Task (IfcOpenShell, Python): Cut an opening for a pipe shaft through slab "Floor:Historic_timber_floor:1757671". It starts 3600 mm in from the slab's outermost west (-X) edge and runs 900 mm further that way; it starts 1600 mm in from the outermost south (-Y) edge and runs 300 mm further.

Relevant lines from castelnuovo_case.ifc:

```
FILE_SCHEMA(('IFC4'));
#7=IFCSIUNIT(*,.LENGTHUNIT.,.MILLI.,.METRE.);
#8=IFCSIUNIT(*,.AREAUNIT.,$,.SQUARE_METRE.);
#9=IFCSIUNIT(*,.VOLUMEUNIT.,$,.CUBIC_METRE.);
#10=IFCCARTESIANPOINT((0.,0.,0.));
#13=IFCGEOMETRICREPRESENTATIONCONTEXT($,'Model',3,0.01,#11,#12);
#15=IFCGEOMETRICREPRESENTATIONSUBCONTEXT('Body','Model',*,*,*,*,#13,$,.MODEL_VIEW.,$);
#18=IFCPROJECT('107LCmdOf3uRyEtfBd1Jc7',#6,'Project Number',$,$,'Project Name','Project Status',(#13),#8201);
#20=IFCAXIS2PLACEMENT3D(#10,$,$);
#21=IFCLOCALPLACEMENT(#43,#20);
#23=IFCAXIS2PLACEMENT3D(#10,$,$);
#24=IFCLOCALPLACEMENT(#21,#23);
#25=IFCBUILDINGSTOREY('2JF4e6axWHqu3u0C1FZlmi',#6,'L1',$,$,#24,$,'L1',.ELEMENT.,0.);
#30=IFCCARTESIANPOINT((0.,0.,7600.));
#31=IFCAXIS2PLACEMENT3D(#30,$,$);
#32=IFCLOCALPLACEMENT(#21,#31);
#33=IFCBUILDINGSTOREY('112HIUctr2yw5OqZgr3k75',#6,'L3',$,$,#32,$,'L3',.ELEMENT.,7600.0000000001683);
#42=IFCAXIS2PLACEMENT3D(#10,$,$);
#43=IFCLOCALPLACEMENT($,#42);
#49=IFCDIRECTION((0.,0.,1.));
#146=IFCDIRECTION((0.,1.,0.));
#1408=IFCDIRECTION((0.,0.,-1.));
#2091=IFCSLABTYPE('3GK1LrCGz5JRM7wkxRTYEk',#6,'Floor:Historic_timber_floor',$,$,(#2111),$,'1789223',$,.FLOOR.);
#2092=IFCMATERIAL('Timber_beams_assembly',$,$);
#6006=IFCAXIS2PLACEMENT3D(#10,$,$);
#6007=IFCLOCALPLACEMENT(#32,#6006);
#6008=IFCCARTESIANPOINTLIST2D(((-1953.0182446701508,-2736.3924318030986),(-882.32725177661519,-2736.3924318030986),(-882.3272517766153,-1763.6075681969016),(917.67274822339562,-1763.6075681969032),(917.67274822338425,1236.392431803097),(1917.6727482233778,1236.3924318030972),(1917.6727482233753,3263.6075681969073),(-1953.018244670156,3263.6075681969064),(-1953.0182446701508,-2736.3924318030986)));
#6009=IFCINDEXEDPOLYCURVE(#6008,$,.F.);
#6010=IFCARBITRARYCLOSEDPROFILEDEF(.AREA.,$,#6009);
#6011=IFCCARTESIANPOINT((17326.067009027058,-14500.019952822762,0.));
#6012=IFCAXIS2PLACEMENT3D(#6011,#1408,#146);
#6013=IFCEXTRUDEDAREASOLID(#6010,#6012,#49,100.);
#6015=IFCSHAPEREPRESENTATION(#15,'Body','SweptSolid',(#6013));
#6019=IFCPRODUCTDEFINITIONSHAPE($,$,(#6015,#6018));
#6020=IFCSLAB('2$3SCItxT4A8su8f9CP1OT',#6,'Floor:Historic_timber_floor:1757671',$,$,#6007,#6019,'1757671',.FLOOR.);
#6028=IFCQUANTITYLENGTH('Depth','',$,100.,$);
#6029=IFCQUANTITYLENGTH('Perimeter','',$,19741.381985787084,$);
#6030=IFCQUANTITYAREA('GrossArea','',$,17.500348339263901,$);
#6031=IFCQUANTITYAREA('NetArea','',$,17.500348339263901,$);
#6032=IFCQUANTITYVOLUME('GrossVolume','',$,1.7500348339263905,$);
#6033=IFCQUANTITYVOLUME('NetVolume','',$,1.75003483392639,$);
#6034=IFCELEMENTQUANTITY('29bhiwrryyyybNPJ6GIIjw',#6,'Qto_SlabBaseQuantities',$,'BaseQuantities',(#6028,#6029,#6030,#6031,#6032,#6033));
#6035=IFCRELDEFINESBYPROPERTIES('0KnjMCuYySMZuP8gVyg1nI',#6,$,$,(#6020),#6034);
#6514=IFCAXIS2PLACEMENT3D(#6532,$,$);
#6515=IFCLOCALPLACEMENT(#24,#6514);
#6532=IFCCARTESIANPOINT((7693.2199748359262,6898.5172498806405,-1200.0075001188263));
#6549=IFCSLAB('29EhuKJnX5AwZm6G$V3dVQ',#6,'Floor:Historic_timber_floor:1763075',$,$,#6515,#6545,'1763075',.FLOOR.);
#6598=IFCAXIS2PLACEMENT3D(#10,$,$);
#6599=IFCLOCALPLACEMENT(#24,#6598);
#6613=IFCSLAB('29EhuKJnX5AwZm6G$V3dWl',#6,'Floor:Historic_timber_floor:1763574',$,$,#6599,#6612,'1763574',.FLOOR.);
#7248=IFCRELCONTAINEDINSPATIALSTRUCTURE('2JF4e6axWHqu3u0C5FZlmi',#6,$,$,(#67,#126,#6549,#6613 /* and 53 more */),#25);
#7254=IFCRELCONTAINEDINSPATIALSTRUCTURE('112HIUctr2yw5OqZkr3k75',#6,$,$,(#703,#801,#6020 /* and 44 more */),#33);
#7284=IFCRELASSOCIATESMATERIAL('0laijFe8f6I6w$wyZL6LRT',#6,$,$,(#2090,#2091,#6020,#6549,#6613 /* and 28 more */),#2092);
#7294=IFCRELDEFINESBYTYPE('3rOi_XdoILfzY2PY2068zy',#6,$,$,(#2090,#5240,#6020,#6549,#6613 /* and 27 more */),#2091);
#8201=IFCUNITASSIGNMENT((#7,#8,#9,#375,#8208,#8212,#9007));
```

```python
import numpy as np
import ifcopenshell
import ifcopenshell.api.feature
import ifcopenshell.api.geometry
import ifcopenshell.api.pset
import ifcopenshell.api.root
import ifcopenshell.geom
import ifcopenshell.util.element
import ifcopenshell.util.placement
import ifcopenshell.util.representation
import ifcopenshell.util.shape
import ifcopenshell.util.unit

model = ifcopenshell.open("castelnuovo_case.ifc")
unit_scale = ifcopenshell.util.unit.calculate_unit_scale(model)
area_scale = ifcopenshell.util.unit.calculate_unit_scale(model, "AREAUNIT")
volume_scale = ifcopenshell.util.unit.calculate_unit_scale(model, "VOLUMEUNIT")
settings = ifcopenshell.geom.settings()


def volume(element):
    """Net volume in cubic metres, openings subtracted."""
    shape = ifcopenshell.geom.create_shape(settings, element)
    return ifcopenshell.util.shape.get_volume(shape.geometry)


slab = model.by_guid("2$3SCItxT4A8su8f9CP1OT")
before = volume(slab)

# Extent in the slab's own axes, in metres. The edges named are its -X and -Y sides.
slab_shape = ifcopenshell.geom.create_shape(settings, slab)
vertices = ifcopenshell.util.shape.get_vertices(slab_shape.geometry)
x_min, y_min, bottom = vertices.min(axis=0)
top = vertices[:, 2].max()

opening = ifcopenshell.api.root.create_entity(model, ifc_class="IfcOpeningElement", name="Pipe shaft opening", predefined_type="OPENING")
context = ifcopenshell.util.representation.get_context(model, "Model", "Body", "MODEL_VIEW")
width, depth = 0.9, 0.3
outline = [(0.0, 0.0), (width, 0.0), (width, depth), (0.0, depth), (0.0, 0.0)]
# Overshoot both faces by 50 mm so the cut is clean.
shape = ifcopenshell.api.geometry.add_slab_representation(
    model, context=context, depth=top - bottom + 0.1, polyline=outline
)
ifcopenshell.api.geometry.assign_representation(model, product=opening, representation=shape)

matrix = ifcopenshell.util.placement.get_local_placement(slab.ObjectPlacement)
matrix[:, 3] = matrix @ np.append(np.array([x_min + 3.6, y_min + 1.6, bottom - 0.05]) / unit_scale, 1.0)
ifcopenshell.api.geometry.edit_object_placement(model, product=opening, matrix=matrix, is_si=False)
ifcopenshell.api.feature.add_feature(model, feature=opening, element=slab)

after = volume(slab)

# Update the slab's stored quantities.
qto = model.by_id(ifcopenshell.util.element.get_pset(slab, "Qto_SlabBaseQuantities", should_inherit=False)["id"])
ifcopenshell.api.pset.edit_qto(model, qto=qto, properties={
    "NetArea": after / (top - bottom) / area_scale,
    "NetVolume": after / volume_scale,
})

print(f"slab volume {before:.3f} -> {after:.3f} m3")

model.write("castelnuovo_case_rev.ifc")
```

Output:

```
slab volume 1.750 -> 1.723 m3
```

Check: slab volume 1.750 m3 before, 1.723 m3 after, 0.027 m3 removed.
